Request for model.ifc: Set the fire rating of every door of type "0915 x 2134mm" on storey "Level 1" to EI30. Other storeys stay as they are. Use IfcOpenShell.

First a look at what the model holds.

```python
import ifcopenshell
import ifcopenshell.util.element

model = ifcopenshell.open("model.ifc")
print(model.schema)
storey = next(s for s in model.by_type("IfcBuildingStorey") if s.Name == "Level 1")
doors = [e for e in ifcopenshell.util.element.get_decomposition(storey) if e.is_a("IfcDoor")]
seen = {}
for e in doors:
    element_type = ifcopenshell.util.element.get_type(e)
    key = (element_type.Name if element_type != e and element_type else None, ifcopenshell.util.element.get_pset(e, "Pset_DoorCommon", "FireRating"))
    seen[key] = seen.get(key, 0) + 1
for (name, value), count in sorted(seen.items(), key=str):
    print(count, "x", name, "|", value)
```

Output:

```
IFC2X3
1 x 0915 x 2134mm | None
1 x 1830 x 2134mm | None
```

```python
import ifcopenshell
import ifcopenshell.api.pset
import ifcopenshell.util.element

model = ifcopenshell.open("model.ifc")

storey = next(s for s in model.by_type("IfcBuildingStorey") if s.Name == "Level 1")
doors = [e for e in ifcopenshell.util.element.get_decomposition(storey) if e.is_a("IfcDoor")]

count = 0
for e in doors:
    element_type = ifcopenshell.util.element.get_type(e)
    if element_type in (None, e) or element_type.Name != "0915 x 2134mm":
        continue
    # add_pset returns the element's existing set when there is one.
    pset = ifcopenshell.api.pset.add_pset(model, product=e, name="Pset_DoorCommon")
    ifcopenshell.api.pset.edit_pset(model, pset=pset, properties={"FireRating": "EI30"})
    count += 1

print(count, "doors updated")

model.write("model_updated.ifc")
```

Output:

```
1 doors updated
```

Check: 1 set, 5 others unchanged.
